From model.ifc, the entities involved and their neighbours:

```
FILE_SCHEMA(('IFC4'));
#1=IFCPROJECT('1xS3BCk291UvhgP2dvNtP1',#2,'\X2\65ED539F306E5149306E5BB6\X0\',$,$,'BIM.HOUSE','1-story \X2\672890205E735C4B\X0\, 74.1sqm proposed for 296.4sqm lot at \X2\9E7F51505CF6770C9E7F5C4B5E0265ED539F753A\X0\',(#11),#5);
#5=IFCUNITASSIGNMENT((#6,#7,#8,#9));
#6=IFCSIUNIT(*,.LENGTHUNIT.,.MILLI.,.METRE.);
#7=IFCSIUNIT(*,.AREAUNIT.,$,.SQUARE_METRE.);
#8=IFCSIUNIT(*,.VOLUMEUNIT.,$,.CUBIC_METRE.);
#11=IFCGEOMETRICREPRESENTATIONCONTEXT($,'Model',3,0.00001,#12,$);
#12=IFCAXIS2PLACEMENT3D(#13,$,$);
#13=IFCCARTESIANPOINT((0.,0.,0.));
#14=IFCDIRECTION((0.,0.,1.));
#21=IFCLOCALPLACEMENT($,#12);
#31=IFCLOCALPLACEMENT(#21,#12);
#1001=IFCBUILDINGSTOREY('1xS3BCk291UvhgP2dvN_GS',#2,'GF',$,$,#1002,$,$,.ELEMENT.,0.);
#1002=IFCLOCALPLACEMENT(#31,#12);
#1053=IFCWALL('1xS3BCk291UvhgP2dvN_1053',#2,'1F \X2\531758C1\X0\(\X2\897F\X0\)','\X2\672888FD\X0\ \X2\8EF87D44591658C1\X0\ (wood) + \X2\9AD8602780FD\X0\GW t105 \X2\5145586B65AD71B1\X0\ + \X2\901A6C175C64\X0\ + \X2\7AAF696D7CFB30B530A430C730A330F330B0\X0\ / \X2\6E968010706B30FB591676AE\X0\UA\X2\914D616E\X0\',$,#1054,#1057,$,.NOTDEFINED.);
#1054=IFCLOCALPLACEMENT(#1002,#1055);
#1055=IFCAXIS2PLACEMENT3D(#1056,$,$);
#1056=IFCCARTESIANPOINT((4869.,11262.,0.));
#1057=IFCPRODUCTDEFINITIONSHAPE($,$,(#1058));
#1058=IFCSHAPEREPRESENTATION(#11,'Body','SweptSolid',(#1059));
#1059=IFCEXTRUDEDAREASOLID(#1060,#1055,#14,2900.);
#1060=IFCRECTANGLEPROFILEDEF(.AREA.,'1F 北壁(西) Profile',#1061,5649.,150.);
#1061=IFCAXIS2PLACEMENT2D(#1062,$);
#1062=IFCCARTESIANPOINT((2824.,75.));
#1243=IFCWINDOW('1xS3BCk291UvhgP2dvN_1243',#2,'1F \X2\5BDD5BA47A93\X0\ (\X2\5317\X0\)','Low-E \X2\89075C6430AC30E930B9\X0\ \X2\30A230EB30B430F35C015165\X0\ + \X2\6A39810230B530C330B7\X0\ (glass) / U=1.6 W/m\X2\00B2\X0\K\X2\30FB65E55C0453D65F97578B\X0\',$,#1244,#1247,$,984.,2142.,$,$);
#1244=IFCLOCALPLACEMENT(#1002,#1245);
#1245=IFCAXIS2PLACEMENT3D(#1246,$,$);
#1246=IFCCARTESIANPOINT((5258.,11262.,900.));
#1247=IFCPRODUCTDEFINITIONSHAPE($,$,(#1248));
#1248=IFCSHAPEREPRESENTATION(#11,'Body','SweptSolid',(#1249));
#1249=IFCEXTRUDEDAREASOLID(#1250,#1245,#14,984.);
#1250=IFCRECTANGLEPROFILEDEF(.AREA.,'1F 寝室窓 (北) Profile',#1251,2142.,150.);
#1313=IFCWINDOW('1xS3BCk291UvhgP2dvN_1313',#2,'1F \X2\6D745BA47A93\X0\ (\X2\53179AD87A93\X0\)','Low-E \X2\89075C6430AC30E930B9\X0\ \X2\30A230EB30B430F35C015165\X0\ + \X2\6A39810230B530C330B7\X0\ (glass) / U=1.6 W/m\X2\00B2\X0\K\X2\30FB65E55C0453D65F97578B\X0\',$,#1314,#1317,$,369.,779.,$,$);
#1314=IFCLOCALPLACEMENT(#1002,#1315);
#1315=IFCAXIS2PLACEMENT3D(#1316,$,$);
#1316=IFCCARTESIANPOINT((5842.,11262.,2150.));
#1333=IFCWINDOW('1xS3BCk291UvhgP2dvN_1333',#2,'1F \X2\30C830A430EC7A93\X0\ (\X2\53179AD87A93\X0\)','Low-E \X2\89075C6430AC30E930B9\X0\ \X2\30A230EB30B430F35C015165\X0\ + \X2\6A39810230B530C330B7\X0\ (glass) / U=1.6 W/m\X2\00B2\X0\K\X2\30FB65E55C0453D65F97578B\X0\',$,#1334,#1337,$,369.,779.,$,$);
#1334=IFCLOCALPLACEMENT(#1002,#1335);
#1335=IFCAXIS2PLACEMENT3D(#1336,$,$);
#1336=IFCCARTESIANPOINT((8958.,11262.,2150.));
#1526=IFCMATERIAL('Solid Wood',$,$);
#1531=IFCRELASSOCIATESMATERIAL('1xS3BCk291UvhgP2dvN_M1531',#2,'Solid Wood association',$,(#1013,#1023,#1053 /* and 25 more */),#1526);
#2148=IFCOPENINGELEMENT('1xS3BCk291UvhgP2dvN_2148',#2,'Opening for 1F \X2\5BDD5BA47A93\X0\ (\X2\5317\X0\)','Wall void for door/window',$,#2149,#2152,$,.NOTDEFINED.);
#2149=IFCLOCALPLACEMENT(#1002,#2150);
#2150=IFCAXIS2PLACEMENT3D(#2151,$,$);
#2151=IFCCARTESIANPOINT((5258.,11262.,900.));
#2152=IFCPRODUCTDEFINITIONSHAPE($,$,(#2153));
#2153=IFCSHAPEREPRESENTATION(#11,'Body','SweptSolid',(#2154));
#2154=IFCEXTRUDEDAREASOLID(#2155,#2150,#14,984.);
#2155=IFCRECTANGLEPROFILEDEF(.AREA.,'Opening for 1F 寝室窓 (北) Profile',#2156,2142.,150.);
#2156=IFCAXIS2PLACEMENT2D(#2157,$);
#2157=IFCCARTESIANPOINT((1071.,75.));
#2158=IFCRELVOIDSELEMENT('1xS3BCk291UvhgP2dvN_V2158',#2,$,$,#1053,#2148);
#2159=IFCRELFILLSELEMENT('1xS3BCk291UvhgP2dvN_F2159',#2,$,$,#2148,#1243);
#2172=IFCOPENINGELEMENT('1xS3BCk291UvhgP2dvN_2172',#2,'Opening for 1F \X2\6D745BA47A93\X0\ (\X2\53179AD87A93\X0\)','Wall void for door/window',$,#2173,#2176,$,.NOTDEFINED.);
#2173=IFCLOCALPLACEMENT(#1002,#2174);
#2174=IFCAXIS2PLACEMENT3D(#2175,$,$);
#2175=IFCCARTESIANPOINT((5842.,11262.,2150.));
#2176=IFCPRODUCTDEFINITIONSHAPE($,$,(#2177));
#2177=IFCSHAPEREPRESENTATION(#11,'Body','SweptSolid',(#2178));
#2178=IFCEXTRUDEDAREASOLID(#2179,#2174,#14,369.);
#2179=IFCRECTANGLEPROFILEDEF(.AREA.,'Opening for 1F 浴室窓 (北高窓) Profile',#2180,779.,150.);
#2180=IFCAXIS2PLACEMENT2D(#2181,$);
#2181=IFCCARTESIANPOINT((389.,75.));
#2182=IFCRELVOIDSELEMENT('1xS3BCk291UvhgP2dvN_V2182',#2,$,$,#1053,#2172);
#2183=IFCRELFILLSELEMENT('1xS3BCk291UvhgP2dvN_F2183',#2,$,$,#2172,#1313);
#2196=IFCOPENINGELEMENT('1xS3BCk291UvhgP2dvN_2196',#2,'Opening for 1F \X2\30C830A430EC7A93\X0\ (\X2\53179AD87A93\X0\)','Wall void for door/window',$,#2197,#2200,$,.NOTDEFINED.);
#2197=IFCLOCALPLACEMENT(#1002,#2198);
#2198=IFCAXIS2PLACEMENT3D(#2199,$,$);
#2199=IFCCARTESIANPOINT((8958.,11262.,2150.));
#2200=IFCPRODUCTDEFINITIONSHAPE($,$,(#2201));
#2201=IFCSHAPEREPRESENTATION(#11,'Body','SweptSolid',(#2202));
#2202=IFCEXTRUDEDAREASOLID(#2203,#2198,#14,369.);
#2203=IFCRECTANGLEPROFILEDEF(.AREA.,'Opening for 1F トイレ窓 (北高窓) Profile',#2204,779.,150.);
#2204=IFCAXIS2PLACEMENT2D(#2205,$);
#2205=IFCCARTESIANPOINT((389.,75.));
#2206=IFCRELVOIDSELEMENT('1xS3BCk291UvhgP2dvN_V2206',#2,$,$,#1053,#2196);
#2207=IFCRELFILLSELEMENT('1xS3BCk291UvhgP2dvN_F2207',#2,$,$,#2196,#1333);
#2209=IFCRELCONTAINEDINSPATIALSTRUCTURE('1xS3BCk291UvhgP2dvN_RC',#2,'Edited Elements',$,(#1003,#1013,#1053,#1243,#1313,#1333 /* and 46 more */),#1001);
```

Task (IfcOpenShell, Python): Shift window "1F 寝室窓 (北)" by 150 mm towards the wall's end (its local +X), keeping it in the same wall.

```python
import ifcopenshell
import ifcopenshell.api.geometry
import ifcopenshell.util.placement
import ifcopenshell.util.unit

model = ifcopenshell.open("model.ifc")
unit_scale = ifcopenshell.util.unit.calculate_unit_scale(model)

window = model.by_guid("1xS3BCk291UvhgP2dvN_1243")
opening = window.FillsVoids[0].RelatingOpeningElement
wall = opening.VoidsElements[0].RelatingBuildingElement

wall_matrix = ifcopenshell.util.placement.get_local_placement(wall.ObjectPlacement)
shift = wall_matrix[:3, 0] * 0.15 / unit_scale
before = ifcopenshell.util.placement.get_local_placement(window.ObjectPlacement)[:3, 3].copy()

# The window is not placed relative to its opening, so move both.
for product in (opening, window):
    matrix = ifcopenshell.util.placement.get_local_placement(product.ObjectPlacement)
    matrix[:3, 3] += shift
    ifcopenshell.api.geometry.edit_object_placement(model, product=product, matrix=matrix, is_si=False)

after = ifcopenshell.util.placement.get_local_placement(window.ObjectPlacement)[:3, 3]
print("window moved by", (after - before).round(3) + 0.0)

model.write("model_rev.ifc")
```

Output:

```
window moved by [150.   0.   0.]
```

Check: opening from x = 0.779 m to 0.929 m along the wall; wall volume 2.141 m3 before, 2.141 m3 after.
